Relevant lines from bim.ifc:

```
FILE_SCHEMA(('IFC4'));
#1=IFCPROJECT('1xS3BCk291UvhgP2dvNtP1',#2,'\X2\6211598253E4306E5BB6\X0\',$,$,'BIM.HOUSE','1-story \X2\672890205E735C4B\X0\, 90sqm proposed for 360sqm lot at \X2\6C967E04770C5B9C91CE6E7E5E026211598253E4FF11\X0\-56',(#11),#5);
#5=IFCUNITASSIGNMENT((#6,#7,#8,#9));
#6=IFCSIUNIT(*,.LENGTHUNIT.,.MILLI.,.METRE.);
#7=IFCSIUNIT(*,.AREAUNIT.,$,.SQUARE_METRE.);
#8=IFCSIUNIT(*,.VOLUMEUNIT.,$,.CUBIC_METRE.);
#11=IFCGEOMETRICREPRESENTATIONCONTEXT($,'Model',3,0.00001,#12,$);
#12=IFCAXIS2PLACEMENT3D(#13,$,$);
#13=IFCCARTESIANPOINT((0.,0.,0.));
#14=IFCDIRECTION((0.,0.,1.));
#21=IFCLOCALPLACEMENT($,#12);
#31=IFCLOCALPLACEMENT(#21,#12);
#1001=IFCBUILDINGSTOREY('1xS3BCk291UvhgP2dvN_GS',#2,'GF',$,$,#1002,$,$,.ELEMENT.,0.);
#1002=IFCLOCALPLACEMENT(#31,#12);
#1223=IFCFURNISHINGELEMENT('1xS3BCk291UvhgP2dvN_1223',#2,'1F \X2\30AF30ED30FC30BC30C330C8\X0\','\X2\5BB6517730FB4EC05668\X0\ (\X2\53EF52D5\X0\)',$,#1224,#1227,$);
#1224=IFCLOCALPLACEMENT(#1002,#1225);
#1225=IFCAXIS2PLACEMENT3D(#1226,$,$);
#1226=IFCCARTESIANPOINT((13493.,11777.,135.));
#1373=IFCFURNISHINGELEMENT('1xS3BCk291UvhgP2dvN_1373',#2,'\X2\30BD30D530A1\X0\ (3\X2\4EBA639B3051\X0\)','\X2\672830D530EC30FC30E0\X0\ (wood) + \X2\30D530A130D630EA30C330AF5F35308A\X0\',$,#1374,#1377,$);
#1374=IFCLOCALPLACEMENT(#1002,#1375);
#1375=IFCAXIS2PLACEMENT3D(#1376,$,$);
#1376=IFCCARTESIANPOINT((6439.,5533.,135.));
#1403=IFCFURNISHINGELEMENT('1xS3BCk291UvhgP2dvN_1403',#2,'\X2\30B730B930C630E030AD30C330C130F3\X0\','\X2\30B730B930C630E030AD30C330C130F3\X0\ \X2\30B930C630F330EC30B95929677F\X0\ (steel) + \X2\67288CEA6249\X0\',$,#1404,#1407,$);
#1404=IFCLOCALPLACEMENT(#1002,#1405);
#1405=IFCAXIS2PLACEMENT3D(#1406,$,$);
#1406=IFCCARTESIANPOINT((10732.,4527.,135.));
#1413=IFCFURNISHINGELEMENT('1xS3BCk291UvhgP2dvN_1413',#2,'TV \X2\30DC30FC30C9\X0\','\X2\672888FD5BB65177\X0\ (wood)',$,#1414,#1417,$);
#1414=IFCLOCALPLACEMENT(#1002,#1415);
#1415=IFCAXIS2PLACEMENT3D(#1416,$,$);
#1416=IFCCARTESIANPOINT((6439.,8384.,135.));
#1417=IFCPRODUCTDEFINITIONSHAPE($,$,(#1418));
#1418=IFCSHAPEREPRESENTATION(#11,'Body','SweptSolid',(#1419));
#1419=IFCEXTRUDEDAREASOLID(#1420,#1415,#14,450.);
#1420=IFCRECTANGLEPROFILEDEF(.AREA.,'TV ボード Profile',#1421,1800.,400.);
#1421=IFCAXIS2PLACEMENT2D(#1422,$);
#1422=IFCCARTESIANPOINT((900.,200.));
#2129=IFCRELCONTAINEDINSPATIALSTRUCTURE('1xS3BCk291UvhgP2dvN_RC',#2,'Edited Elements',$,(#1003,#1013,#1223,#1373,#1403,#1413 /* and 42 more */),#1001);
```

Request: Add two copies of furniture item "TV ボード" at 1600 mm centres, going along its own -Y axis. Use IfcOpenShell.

```python
import ifcopenshell
import ifcopenshell.api.geometry
import ifcopenshell.api.root
import ifcopenshell.util.element
import ifcopenshell.util.placement

model = ifcopenshell.open("bim.ifc")


def reuse_history(source, copy):
    """copy_class also copies each property set's owner history, people and application; keep the originals."""
    for rel in copy.IsDefinedBy:
        if rel.is_a("IfcRelDefinesByProperties") and (history := rel.RelatingPropertyDefinition.OwnerHistory):
            rel.RelatingPropertyDefinition.OwnerHistory = source.OwnerHistory
            ifcopenshell.util.element.remove_deep2(model, history)


source = model.by_guid("1xS3BCk291UvhgP2dvN_1413")
base = ifcopenshell.util.placement.get_local_placement(source.ObjectPlacement)
step = -base[:3, 1] * 1600.0

for i in range(1, 3):
    copy = ifcopenshell.api.root.copy_class(model, product=source)
    copy.Representation = ifcopenshell.util.element.copy_deep(
        model, source.Representation, exclude=["IfcGeometricRepresentationContext", "IfcRepresentationMap"]
    )
    reuse_history(source, copy)
    matrix = base.copy()
    matrix[:3, 3] += i * step
    print("added at", matrix[:3, 3].round(3) + 0.0)
    ifcopenshell.api.geometry.edit_object_placement(model, product=copy, matrix=matrix, is_si=False)

model.write("bim_v2.ifc")
```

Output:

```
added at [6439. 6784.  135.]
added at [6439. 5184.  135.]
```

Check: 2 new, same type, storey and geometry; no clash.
